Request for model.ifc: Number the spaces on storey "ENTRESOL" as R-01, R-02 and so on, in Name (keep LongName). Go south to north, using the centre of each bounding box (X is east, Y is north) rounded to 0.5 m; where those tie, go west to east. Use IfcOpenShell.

First a look at what the model holds.

```python
import ifcopenshell
import ifcopenshell.util.element
import ifcopenshell.util.placement

model = ifcopenshell.open("model.ifc")
print(model.schema)
storey = next(s for s in model.by_type("IfcBuildingStorey") if s.Name == "ENTRESOL")
spaces = [e for e in ifcopenshell.util.element.get_decomposition(storey) if e.is_a("IfcSpace")]
for e in sorted(spaces, key=lambda e: e.id()):
    origin = ifcopenshell.util.placement.get_local_placement(e.ObjectPlacement)[:3, 3]
    print(e.id(), e.Name, e.LongName, origin.round(2) + 0.0, sep=" | ")
```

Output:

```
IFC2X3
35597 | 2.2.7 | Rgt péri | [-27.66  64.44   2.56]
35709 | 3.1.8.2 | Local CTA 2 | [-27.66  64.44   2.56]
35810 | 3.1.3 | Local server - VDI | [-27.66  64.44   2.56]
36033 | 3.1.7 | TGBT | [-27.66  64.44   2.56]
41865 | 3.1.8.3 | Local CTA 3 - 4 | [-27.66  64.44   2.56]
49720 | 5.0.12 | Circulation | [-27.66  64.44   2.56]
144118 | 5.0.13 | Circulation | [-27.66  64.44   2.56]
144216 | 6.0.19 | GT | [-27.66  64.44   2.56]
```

```python
import ifcopenshell
import ifcopenshell.geom
import ifcopenshell.util.element
import ifcopenshell.util.shape

model = ifcopenshell.open("model.ifc")
settings = ifcopenshell.geom.settings()
settings.set("use-world-coords", True)


def centre(element):
    shape = ifcopenshell.geom.create_shape(settings, element)
    return ifcopenshell.util.shape.get_bbox_centroid(shape.geometry)


storey = next(s for s in model.by_type("IfcBuildingStorey") if s.Name == "ENTRESOL")
spaces = [e for e in ifcopenshell.util.element.get_decomposition(storey) if e.is_a("IfcSpace")]

# Insertion points can sit at a corner or the storey origin, so sort by the geometry (in metres).
centres = {e: centre(e) for e in spaces}
spaces.sort(key=lambda e: (round(centres[e][1] / 0.5), centres[e][0]))

for i, e in enumerate(spaces, start=1):
    number = f"R-{i:02d}"
    e.Name = number
    print(e.id(), number)

model.write("model_rev.ifc")
```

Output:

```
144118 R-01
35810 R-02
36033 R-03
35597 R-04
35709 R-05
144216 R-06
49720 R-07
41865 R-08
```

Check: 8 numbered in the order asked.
